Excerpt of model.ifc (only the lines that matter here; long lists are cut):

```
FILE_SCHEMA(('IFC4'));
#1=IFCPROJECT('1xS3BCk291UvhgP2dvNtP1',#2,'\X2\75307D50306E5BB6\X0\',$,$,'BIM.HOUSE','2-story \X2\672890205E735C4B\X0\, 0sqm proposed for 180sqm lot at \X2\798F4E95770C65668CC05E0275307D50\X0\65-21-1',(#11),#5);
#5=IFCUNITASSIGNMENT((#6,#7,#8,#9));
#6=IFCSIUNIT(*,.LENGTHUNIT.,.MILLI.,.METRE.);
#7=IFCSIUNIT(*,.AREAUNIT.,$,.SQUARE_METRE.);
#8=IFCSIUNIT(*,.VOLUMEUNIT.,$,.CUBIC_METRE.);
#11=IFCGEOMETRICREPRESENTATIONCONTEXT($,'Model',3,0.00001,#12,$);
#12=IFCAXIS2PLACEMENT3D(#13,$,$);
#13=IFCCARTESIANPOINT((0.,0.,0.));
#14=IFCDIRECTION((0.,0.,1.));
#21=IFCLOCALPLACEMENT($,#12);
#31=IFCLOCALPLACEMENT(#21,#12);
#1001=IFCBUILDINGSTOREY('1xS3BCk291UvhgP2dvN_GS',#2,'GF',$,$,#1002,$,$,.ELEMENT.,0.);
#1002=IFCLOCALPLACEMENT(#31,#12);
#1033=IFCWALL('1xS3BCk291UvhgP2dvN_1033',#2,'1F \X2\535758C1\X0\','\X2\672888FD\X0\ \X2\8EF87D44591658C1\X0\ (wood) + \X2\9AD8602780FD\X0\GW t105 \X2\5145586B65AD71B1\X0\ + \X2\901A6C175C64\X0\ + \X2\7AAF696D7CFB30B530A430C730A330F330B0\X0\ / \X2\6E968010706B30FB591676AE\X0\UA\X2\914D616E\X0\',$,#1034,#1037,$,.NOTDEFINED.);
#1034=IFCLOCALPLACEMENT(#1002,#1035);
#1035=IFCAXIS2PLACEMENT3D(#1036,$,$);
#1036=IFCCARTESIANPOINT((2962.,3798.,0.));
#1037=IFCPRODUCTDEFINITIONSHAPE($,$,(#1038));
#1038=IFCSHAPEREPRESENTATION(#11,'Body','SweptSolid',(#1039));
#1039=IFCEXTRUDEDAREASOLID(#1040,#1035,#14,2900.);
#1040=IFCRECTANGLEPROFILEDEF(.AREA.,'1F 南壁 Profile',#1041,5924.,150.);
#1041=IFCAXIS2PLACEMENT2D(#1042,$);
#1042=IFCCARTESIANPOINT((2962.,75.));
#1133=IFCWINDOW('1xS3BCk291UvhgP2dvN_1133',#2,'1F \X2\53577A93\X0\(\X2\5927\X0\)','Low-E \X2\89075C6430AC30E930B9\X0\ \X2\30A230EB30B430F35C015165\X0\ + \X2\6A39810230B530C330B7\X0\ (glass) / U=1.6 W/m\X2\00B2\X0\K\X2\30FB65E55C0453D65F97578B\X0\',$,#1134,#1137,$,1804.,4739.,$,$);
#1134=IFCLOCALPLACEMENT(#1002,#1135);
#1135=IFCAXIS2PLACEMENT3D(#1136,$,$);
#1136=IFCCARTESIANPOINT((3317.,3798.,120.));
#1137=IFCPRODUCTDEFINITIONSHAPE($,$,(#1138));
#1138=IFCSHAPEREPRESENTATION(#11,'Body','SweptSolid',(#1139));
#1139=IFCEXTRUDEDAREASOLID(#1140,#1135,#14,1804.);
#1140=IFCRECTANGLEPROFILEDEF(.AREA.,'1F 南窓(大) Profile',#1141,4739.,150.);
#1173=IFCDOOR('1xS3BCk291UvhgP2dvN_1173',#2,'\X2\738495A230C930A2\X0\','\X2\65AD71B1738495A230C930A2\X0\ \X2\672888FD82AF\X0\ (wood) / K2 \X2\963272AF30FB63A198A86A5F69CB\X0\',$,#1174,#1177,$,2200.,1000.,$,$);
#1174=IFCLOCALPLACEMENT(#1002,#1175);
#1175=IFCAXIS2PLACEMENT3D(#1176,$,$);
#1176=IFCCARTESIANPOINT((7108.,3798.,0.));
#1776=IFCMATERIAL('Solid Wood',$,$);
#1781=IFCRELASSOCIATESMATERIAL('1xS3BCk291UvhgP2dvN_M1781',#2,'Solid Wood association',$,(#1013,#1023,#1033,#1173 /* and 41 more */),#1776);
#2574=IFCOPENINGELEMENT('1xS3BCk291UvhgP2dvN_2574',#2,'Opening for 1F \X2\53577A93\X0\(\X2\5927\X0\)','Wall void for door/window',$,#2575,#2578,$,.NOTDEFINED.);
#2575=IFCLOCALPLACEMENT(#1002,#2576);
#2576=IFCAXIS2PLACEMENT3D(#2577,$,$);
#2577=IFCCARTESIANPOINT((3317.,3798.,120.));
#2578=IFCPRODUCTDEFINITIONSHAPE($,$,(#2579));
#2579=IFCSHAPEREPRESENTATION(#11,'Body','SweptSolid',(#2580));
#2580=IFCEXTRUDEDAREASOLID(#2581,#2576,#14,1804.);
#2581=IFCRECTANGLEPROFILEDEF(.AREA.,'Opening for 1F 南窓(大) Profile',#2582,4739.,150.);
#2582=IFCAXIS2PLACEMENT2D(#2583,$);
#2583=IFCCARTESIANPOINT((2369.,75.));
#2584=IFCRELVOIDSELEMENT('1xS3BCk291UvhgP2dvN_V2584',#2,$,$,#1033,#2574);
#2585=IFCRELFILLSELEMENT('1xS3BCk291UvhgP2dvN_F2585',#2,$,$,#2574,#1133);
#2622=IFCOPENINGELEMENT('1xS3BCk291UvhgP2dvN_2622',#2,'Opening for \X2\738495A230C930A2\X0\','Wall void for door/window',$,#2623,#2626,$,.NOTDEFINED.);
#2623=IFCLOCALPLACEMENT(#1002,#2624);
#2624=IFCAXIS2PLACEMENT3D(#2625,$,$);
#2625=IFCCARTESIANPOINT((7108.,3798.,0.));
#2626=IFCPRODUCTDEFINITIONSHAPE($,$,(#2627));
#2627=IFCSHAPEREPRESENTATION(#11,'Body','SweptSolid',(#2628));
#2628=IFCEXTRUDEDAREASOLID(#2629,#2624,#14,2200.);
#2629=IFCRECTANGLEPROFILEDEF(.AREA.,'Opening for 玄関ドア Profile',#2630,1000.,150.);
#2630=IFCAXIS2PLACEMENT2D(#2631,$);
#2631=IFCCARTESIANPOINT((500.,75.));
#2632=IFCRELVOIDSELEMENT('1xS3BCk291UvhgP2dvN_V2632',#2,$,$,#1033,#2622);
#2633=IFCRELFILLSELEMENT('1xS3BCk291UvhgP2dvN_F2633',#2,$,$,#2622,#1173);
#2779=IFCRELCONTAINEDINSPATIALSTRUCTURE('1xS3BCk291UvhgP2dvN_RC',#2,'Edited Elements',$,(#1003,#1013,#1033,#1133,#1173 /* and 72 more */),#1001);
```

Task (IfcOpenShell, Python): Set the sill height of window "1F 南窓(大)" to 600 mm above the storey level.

```python
import numpy as np
import ifcopenshell
import ifcopenshell.api.geometry
import ifcopenshell.geom
import ifcopenshell.util.element
import ifcopenshell.util.placement
import ifcopenshell.util.shape
import ifcopenshell.util.unit

model = ifcopenshell.open("model.ifc")
unit_scale = ifcopenshell.util.unit.calculate_unit_scale(model)

window = model.by_id(1133)
opening = window.FillsVoids[0].RelatingOpeningElement
storey = ifcopenshell.util.element.get_container(window, ifc_class="IfcBuildingStorey")
level = ifcopenshell.util.placement.get_local_placement(storey.ObjectPlacement)[2, 3]

# The opening's origin need not be at the sill, so measure its lowest point.
shape = ifcopenshell.geom.create_shape(ifcopenshell.geom.settings(), opening)
bottom = ifcopenshell.util.shape.get_shape_bottom_elevation(shape, shape.geometry) / unit_scale
dz = level + 0.6 / unit_scale - bottom

shift = np.array([0.0, 0.0, dz])
# The window is not placed relative to its opening, so move both.
for product in (opening, window):
    matrix = ifcopenshell.util.placement.get_local_placement(product.ObjectPlacement)
    matrix[:3, 3] += shift
    ifcopenshell.api.geometry.edit_object_placement(model, product=product, matrix=matrix, is_si=False)

print(f"moved by {dz * unit_scale:+.3f} m")

model.write("model_updated.ifc")
```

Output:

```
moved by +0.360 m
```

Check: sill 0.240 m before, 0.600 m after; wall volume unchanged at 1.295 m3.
